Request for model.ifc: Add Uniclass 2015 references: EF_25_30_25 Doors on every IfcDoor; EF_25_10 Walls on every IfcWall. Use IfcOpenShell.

First a look at what the model holds.

```python
import ifcopenshell

model = ifcopenshell.open("model.ifc")
print(model.schema)
print("classifications:", [c.Name for c in model.by_type("IfcClassification")])
for ifc_class in ("IfcDoor", "IfcRoof", "IfcStair", "IfcWall", "IfcWindow"):
    print(ifc_class, len(model.by_type(ifc_class)))
```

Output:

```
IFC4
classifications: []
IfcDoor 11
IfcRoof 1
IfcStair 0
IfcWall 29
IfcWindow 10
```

```python
import ifcopenshell
import ifcopenshell.api.classification

model = ifcopenshell.open("model.ifc")

system = ifcopenshell.api.classification.add_classification(model, classification="Uniclass 2015")

codes = {
    "IfcDoor": ("EF_25_30_25", "Doors"),
    "IfcWall": ("EF_25_10", "Walls"),
}
for ifc_class, (code, name) in codes.items():
    products = model.by_type(ifc_class)
    ifcopenshell.api.classification.add_reference(
        model, products=products, classification=system, identification=code, name=name
    )
    print(code, len(products))

model.write("model-out.ifc")
```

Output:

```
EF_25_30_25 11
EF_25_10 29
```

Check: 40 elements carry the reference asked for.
